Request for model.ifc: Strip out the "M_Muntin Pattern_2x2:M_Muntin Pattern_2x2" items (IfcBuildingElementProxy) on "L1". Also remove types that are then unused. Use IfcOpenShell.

First a look at what the model holds.

```python
import ifcopenshell
import ifcopenshell.util.element

model = ifcopenshell.open("model.ifc")
print(model.schema)
storey = next(s for s in model.by_type("IfcBuildingStorey") if s.Name == "L1")
proxies = [e for e in ifcopenshell.util.element.get_decomposition(storey) if e.is_a("IfcBuildingElementProxy")]
seen = {}
for e in proxies:
    element_type = ifcopenshell.util.element.get_type(e)
    name = element_type.Name if element_type not in (None, e) else None
    seen[name] = seen.get(name, 0) + 1
for name, count in sorted(seen.items(), key=str):
    print(count, "x", name)
```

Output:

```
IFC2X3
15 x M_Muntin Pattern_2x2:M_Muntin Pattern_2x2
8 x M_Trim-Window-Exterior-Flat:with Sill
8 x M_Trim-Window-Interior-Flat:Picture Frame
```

```python
import ifcopenshell
import ifcopenshell.api.root
import ifcopenshell.util.element

model = ifcopenshell.open("model.ifc")

storey = next(s for s in model.by_type("IfcBuildingStorey") if s.Name == "L1")
proxies = [e for e in ifcopenshell.util.element.get_decomposition(storey) if e.is_a("IfcBuildingElementProxy")]
targets = [e for e in proxies if (t := ifcopenshell.util.element.get_type(e)) not in (None, e) and t.Name == "M_Muntin Pattern_2x2:M_Muntin Pattern_2x2"]
types = {ifcopenshell.util.element.get_type(e) for e in targets} - {None, *targets}

for e in targets:
    ifcopenshell.api.root.remove_product(model, product=e)
print(len(targets), "removed")

unused = [t for t in types if not ifcopenshell.util.element.get_types(t)]
for t in unused:
    ifcopenshell.api.root.remove_product(model, product=t)
print(len(unused), "unused types removed")

model.write("model_edited.ifc")
```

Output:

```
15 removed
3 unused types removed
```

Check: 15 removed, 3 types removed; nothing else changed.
